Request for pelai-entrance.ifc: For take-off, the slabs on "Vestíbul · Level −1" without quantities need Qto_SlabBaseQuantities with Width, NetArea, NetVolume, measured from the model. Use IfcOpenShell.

First a look at what the model holds.

```python
import ifcopenshell
import ifcopenshell.util.element
import ifcopenshell.util.unit

model = ifcopenshell.open("pelai-entrance.ifc")
print(model.schema)
for unit_type in ("LENGTHUNIT", "AREAUNIT", "VOLUMEUNIT"):
    print(unit_type, ifcopenshell.util.unit.calculate_unit_scale(model, unit_type))
storey = next(s for s in model.by_type("IfcBuildingStorey") if s.Name == "Vestíbul · Level −1")
slabs = [e for e in ifcopenshell.util.element.get_decomposition(storey) if e.is_a("IfcSlab")]
for e in sorted(slabs, key=lambda e: e.id()):
    print(e.id(), e.is_a(), e.Name, list(ifcopenshell.util.element.get_psets(e, qtos_only=True)), sep=" | ")
```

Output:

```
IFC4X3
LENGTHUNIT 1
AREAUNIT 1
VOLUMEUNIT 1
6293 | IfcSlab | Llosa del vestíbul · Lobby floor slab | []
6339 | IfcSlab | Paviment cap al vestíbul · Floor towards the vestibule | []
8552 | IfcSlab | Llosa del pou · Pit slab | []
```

```python
import ifcopenshell
import ifcopenshell.api.pset
import ifcopenshell.geom
import ifcopenshell.util.element
import ifcopenshell.util.shape
import ifcopenshell.util.unit

model = ifcopenshell.open("pelai-entrance.ifc")
unit_scale = ifcopenshell.util.unit.calculate_unit_scale(model)
area_scale = ifcopenshell.util.unit.calculate_unit_scale(model, "AREAUNIT")
volume_scale = ifcopenshell.util.unit.calculate_unit_scale(model, "VOLUMEUNIT")
settings = ifcopenshell.geom.settings()

storey = next(s for s in model.by_type("IfcBuildingStorey") if s.Name == "Vestíbul · Level −1")
slabs = [e for e in ifcopenshell.util.element.get_decomposition(storey) if e.is_a("IfcSlab")]

for e in sorted(slabs, key=lambda e: e.id()):
    if ifcopenshell.util.element.get_psets(e, qtos_only=True, should_inherit=False):
        continue
    # Geometry comes back in metres, in the element's own axes.
    shape = ifcopenshell.geom.create_shape(settings, e)
    values = {
        "Width": ifcopenshell.util.shape.get_z(shape.geometry) / unit_scale,
        "NetArea": ifcopenshell.util.shape.get_footprint_area(shape.geometry) / area_scale,
        "NetVolume": ifcopenshell.util.shape.get_volume(shape.geometry) / volume_scale,
    }
    qto = ifcopenshell.api.pset.add_qto(model, product=e, name="Qto_SlabBaseQuantities")
    ifcopenshell.api.pset.edit_qto(model, qto=qto, properties=values)
    print(e.id(), {k: round(v, 3) for k, v in values.items()})

model.write("pelai-entrance-out.ifc")
```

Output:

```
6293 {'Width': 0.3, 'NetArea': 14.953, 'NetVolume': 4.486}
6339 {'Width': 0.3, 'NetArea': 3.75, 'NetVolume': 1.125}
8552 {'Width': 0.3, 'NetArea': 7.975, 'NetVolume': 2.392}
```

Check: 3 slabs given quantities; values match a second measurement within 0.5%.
